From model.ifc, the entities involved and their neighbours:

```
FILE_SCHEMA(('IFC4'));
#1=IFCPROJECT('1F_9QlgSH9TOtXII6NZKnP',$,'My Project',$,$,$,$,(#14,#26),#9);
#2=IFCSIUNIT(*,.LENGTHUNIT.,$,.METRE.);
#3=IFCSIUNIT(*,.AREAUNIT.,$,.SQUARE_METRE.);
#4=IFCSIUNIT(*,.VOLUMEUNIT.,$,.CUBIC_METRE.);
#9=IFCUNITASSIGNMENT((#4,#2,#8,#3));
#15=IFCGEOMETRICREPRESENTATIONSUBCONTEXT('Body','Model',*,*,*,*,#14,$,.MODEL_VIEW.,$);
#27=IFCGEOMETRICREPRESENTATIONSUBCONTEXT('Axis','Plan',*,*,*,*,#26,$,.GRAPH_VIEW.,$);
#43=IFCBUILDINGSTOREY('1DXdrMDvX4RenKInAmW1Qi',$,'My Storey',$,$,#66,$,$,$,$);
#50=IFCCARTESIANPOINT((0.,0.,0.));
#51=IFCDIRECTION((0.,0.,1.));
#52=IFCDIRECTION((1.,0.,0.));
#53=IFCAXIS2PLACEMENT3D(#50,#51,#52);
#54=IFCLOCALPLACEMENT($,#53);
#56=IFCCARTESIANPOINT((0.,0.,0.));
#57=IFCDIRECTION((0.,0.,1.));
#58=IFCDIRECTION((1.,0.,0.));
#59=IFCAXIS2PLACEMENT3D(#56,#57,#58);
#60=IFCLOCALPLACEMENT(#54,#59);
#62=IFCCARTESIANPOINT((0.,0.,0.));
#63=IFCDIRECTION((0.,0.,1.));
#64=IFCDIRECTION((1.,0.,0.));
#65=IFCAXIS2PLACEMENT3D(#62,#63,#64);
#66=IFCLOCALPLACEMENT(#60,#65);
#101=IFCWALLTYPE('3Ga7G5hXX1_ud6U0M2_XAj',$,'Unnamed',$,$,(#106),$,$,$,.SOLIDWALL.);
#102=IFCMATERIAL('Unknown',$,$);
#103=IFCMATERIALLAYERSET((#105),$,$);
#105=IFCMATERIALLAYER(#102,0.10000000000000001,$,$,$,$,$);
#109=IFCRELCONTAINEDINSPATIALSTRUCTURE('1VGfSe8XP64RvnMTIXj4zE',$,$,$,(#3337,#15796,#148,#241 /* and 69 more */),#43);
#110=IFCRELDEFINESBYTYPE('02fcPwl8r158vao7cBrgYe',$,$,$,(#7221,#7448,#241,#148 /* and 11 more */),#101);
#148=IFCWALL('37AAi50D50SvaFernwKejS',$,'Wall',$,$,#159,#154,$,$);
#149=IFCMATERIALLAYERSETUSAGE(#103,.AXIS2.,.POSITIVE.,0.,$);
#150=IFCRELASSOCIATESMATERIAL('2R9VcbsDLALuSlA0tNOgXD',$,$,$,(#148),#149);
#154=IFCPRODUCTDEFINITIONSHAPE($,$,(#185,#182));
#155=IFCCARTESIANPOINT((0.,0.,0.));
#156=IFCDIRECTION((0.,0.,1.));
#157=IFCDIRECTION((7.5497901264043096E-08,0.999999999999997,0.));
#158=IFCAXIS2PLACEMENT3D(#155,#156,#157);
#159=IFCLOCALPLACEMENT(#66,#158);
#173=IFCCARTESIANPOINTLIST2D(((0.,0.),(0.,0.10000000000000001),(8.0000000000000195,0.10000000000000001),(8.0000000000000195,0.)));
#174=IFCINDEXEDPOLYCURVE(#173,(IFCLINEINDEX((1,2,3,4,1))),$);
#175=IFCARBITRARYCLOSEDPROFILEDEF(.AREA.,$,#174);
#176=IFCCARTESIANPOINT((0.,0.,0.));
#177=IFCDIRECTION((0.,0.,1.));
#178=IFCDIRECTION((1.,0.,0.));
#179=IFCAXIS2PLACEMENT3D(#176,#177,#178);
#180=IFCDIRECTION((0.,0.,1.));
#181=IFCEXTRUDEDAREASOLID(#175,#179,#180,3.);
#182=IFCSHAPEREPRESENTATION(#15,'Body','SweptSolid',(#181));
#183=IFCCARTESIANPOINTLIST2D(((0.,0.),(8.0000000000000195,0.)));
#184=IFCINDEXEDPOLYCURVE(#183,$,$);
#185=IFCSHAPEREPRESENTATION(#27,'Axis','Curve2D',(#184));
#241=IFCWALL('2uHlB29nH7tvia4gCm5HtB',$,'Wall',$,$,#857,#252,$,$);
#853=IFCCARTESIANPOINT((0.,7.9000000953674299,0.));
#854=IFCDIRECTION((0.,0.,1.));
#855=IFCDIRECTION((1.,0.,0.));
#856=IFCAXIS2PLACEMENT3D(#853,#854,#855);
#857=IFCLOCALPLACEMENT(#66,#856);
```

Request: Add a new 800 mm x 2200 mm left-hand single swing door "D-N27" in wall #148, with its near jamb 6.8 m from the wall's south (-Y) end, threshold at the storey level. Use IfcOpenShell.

```python
import numpy as np
import ifcopenshell
import ifcopenshell.api.feature
import ifcopenshell.api.geometry
import ifcopenshell.api.root
import ifcopenshell.api.spatial
import ifcopenshell.geom
import ifcopenshell.util.element
import ifcopenshell.util.placement
import ifcopenshell.util.representation
import ifcopenshell.util.shape
import ifcopenshell.util.unit

model = ifcopenshell.open("model.ifc")
unit_scale = ifcopenshell.util.unit.calculate_unit_scale(model)
settings = ifcopenshell.geom.settings()


def volume(element):
    """Net volume in cubic metres, openings subtracted."""
    shape = ifcopenshell.geom.create_shape(settings, element)
    return ifcopenshell.util.shape.get_volume(shape.geometry)


wall = model.by_guid("37AAi50D50SvaFernwKejS")
storey = ifcopenshell.util.element.get_container(wall, ifc_class="IfcBuildingStorey")
context = ifcopenshell.util.representation.get_context(model, "Model", "Body", "MODEL_VIEW")
before = volume(wall)

width, height, from_end, sill = 0.8, 2.2, 6.8, 0.0  # metres

# The wall runs along its own X axis, and the end named is its -X end.
wall_shape = ifcopenshell.geom.create_shape(settings, wall)
x, y, z = ifcopenshell.util.shape.get_vertices(wall_shape.geometry).T
start = x.min() + from_end
face, thickness = float(y.min()), float(y.max() - y.min())
wall_matrix = ifcopenshell.util.placement.get_local_placement(wall.ObjectPlacement)
level = ifcopenshell.util.placement.get_local_placement(storey.ObjectPlacement)[2, 3]


def in_wall(x, y):
    """Placement at x, y metres in the wall's axes, at sill height."""
    matrix = wall_matrix.copy()
    matrix[:, 3] = wall_matrix @ np.array([x / unit_scale, y / unit_scale, 0.0, 1.0])
    matrix[2, 3] = level + sill / unit_scale
    return matrix


# Opening: a box that overshoots both wall faces by 50 mm.
opening = ifcopenshell.api.root.create_entity(model, ifc_class="IfcOpeningElement", predefined_type="OPENING")
box = ifcopenshell.api.geometry.add_wall_representation(
    model, context=context, length=width, height=height, thickness=thickness + 0.1
)
ifcopenshell.api.geometry.assign_representation(model, product=opening, representation=box)
ifcopenshell.api.geometry.edit_object_placement(model, product=opening, matrix=in_wall(start, face - 0.05), is_si=False)
ifcopenshell.api.feature.add_feature(model, feature=opening, element=wall)

door = ifcopenshell.api.root.create_entity(model, ifc_class="IfcDoor", name="D-N27", predefined_type="DOOR")
door.OverallWidth, door.OverallHeight = width / unit_scale, height / unit_scale
door.OperationType = "SINGLE_SWING_LEFT"
body = ifcopenshell.api.geometry.add_door_representation(
    model,
    context=context,
    overall_width=door.OverallWidth,
    overall_height=door.OverallHeight,
    operation_type="SINGLE_SWING_LEFT",
    lining_properties={"LiningDepth": thickness / unit_scale, "ThresholdDepth": thickness / unit_scale},
)
ifcopenshell.api.geometry.assign_representation(model, product=door, representation=body)
ifcopenshell.api.spatial.assign_container(model, products=[door], relating_structure=storey)
ifcopenshell.api.feature.add_filling(model, opening=opening, element=door)

# The lining spans the wall, so the door starts at the wall face.
ifcopenshell.api.geometry.edit_object_placement(model, product=door, matrix=in_wall(start, face), is_si=False)

after = volume(wall)

print(f"wall volume {before:.3f} -> {after:.3f} m3")

model.write("model-out.ifc")
```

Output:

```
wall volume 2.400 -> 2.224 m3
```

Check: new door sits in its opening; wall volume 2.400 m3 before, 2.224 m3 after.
